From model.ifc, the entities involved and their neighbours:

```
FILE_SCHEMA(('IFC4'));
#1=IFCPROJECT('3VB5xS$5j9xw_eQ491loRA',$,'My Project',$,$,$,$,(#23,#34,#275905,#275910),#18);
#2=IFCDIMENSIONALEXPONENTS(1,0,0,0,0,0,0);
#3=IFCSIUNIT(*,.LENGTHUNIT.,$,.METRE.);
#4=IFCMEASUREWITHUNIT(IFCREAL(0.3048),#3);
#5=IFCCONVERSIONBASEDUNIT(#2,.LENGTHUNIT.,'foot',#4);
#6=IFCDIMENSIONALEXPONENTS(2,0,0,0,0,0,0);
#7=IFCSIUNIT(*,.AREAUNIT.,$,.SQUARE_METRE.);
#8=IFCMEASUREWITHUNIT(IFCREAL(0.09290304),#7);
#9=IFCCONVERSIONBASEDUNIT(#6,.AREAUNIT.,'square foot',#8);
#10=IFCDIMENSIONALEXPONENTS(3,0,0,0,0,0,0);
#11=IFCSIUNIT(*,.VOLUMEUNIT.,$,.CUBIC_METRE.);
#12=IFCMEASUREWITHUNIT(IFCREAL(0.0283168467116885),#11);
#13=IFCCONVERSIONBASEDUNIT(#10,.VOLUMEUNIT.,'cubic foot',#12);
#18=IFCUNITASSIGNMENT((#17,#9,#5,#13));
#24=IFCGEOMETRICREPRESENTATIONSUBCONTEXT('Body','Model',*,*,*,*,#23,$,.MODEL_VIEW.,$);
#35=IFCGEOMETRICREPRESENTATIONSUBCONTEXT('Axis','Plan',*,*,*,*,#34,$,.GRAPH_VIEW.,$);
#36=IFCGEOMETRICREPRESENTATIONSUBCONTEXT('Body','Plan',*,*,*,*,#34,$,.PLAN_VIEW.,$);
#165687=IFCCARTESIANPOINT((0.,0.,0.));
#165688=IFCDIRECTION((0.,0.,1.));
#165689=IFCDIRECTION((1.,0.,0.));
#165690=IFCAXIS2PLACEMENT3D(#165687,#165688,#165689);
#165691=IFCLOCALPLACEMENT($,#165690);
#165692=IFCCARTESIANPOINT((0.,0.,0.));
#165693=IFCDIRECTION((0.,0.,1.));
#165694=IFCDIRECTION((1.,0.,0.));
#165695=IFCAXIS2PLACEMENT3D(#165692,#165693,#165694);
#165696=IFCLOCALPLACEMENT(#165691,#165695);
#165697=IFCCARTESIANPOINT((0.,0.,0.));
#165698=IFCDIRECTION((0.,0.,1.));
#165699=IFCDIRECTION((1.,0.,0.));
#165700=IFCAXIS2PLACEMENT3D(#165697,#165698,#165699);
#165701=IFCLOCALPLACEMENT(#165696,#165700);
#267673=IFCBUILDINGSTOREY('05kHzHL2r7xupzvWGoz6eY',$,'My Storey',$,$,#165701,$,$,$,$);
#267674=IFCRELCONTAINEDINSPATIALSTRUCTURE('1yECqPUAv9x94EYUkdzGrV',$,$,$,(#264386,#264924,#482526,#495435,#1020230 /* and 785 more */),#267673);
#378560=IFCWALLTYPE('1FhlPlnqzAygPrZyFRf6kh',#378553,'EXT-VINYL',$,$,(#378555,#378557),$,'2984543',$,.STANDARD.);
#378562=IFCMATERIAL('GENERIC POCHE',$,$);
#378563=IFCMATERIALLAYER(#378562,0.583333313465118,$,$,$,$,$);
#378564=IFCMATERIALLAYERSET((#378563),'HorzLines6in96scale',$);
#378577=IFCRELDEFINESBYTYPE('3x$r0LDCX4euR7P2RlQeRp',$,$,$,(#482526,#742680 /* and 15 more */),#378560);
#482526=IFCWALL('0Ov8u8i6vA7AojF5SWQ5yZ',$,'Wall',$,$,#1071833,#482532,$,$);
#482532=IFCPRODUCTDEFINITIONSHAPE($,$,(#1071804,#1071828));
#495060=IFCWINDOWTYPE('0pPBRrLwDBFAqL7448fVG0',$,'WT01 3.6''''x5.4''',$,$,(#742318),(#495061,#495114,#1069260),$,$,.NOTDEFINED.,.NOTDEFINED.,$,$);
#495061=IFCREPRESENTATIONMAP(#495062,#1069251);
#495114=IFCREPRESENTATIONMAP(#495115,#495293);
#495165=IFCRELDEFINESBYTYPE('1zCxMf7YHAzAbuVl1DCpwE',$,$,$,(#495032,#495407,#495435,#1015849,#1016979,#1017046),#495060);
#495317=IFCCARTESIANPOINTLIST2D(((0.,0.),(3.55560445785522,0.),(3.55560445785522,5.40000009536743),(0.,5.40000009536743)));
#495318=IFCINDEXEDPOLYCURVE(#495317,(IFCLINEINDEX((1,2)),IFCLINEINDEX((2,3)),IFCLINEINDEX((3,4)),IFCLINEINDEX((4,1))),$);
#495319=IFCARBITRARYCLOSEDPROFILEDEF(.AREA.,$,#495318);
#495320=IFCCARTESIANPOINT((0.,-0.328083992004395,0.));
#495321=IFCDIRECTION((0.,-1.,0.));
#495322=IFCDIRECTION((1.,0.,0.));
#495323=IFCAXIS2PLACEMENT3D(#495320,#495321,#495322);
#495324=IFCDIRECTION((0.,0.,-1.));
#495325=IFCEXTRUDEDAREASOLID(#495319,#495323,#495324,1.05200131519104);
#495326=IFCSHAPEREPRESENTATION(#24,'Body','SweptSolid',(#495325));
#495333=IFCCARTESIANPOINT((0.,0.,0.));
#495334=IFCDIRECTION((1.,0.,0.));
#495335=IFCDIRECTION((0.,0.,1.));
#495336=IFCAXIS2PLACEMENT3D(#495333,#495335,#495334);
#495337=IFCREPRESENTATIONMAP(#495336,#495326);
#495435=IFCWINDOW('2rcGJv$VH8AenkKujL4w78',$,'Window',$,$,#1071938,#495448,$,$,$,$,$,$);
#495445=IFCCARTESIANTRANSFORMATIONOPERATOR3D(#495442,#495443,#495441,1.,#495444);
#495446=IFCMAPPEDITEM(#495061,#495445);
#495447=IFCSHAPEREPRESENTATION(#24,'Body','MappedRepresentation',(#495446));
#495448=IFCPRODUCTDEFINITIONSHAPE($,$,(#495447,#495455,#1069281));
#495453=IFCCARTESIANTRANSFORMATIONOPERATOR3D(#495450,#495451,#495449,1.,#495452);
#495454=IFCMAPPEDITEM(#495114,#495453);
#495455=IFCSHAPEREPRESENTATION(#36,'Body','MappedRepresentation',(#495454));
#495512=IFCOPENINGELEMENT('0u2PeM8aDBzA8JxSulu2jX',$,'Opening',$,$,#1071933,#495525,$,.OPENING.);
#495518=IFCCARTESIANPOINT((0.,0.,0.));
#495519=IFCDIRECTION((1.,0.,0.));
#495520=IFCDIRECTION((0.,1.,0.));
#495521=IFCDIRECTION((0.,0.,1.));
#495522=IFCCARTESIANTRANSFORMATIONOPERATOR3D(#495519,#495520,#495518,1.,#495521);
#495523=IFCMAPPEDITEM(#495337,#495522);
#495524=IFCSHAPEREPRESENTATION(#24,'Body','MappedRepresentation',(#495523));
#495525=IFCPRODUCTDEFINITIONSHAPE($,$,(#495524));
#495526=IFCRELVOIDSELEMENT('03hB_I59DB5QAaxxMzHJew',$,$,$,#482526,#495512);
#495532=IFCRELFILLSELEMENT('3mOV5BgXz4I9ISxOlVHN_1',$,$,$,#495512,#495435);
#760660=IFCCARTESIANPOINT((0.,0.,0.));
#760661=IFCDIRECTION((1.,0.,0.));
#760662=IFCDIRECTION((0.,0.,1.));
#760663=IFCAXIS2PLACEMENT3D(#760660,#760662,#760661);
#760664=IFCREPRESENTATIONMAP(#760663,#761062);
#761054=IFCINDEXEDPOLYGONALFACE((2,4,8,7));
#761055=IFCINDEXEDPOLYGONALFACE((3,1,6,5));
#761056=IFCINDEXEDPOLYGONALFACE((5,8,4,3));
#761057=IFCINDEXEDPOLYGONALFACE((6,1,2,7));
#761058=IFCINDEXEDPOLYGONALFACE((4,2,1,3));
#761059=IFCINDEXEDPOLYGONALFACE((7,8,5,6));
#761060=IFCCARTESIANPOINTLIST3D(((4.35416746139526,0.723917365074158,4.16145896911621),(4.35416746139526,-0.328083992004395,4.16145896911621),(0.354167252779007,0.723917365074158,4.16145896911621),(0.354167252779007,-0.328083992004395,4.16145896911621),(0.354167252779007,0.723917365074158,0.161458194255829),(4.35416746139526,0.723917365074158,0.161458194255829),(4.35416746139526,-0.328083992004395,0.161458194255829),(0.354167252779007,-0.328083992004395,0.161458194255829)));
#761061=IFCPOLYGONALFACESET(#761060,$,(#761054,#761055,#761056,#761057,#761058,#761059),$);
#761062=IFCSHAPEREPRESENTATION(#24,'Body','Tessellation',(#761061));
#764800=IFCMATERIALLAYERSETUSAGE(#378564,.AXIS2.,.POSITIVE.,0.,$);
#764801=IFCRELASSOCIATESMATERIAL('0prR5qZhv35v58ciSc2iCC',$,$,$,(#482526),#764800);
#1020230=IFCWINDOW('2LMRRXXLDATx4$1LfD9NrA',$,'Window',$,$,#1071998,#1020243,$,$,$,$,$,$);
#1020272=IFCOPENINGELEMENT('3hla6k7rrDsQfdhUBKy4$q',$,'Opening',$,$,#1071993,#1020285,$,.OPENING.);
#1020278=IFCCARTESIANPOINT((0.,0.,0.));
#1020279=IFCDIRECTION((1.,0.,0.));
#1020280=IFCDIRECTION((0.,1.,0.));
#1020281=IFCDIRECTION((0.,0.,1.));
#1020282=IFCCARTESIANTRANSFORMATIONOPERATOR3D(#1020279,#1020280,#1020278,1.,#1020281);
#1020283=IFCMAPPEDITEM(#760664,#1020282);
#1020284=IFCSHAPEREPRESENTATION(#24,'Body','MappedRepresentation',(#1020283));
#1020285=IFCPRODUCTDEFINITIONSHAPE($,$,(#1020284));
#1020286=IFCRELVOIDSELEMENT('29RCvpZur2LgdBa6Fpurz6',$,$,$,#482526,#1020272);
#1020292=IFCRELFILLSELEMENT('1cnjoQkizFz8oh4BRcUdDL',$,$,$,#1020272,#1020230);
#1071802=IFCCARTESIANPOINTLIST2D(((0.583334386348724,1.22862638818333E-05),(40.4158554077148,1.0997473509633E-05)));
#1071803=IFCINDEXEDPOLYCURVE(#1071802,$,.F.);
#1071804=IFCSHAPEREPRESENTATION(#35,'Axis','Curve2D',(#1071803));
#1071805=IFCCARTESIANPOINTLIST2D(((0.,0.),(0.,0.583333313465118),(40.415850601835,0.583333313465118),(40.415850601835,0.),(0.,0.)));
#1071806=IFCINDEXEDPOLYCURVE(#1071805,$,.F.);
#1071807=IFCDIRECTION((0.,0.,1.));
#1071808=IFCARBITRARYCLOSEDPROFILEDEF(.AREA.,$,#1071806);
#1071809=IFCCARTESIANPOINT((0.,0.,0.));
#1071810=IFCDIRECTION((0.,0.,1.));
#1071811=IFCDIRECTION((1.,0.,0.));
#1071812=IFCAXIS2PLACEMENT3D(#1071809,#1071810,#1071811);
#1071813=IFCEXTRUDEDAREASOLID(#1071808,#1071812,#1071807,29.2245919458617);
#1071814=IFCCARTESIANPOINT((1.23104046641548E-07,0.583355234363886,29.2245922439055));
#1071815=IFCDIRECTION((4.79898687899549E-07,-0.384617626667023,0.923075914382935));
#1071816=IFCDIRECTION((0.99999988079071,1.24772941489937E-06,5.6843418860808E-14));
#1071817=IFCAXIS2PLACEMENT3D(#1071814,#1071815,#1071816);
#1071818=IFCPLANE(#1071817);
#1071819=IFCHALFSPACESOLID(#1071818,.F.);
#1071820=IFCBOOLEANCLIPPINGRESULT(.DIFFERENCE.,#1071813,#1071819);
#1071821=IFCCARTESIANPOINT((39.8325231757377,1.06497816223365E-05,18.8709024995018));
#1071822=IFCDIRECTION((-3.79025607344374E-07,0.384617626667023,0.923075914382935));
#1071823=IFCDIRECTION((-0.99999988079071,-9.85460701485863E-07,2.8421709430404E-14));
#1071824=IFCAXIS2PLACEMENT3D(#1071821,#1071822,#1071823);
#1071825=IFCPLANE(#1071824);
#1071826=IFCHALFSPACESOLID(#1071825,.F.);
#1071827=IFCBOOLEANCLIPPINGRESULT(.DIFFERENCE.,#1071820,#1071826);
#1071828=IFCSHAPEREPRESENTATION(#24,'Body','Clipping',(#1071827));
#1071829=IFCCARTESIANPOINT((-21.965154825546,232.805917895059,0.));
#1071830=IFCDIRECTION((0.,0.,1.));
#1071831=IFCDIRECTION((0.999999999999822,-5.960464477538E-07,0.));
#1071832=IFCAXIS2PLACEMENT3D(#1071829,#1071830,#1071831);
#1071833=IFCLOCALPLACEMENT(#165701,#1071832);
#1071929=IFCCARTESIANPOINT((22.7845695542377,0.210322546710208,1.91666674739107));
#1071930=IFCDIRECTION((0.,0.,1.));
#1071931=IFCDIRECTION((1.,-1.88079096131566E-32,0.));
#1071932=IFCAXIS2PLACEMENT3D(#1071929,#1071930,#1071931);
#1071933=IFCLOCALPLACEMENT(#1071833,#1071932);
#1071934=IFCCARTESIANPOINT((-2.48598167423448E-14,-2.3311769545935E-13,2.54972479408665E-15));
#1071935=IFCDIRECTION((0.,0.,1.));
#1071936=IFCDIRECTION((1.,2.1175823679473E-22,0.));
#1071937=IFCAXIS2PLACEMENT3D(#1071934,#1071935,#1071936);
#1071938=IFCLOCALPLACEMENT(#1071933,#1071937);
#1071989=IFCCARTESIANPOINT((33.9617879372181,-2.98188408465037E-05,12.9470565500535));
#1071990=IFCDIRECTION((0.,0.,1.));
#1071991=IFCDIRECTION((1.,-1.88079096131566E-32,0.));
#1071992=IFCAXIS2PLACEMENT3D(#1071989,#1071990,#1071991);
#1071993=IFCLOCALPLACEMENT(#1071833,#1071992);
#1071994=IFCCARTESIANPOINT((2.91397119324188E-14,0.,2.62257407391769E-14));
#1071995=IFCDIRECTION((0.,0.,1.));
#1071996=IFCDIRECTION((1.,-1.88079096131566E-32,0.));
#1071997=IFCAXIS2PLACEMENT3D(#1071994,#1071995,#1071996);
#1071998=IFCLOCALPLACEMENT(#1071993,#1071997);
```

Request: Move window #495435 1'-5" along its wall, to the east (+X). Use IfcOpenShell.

```python
import ifcopenshell
import ifcopenshell.api.geometry
import ifcopenshell.util.placement
import ifcopenshell.util.unit

model = ifcopenshell.open("model.ifc")
unit_scale = ifcopenshell.util.unit.calculate_unit_scale(model)

window = model.by_id(495435)
opening = window.FillsVoids[0].RelatingOpeningElement
wall = opening.VoidsElements[0].RelatingBuildingElement

wall_matrix = ifcopenshell.util.placement.get_local_placement(wall.ObjectPlacement)
shift = wall_matrix[:3, 0] * 17 * 0.0254 / unit_scale
before = ifcopenshell.util.placement.get_local_placement(window.ObjectPlacement)[:3, 3].copy()

# The window is placed relative to its opening, so it follows when the opening moves.
matrix = ifcopenshell.util.placement.get_local_placement(opening.ObjectPlacement)
matrix[:3, 3] += shift
ifcopenshell.api.geometry.edit_object_placement(
    model, product=opening, matrix=matrix, is_si=False, should_transform_children=True
)

after = ifcopenshell.util.placement.get_local_placement(window.ObjectPlacement)[:3, 3]
print("window moved by", (after - before).round(3) + 0.0)

model.write("model-out.ifc")
```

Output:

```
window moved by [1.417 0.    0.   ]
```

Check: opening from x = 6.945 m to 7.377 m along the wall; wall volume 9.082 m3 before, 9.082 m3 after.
